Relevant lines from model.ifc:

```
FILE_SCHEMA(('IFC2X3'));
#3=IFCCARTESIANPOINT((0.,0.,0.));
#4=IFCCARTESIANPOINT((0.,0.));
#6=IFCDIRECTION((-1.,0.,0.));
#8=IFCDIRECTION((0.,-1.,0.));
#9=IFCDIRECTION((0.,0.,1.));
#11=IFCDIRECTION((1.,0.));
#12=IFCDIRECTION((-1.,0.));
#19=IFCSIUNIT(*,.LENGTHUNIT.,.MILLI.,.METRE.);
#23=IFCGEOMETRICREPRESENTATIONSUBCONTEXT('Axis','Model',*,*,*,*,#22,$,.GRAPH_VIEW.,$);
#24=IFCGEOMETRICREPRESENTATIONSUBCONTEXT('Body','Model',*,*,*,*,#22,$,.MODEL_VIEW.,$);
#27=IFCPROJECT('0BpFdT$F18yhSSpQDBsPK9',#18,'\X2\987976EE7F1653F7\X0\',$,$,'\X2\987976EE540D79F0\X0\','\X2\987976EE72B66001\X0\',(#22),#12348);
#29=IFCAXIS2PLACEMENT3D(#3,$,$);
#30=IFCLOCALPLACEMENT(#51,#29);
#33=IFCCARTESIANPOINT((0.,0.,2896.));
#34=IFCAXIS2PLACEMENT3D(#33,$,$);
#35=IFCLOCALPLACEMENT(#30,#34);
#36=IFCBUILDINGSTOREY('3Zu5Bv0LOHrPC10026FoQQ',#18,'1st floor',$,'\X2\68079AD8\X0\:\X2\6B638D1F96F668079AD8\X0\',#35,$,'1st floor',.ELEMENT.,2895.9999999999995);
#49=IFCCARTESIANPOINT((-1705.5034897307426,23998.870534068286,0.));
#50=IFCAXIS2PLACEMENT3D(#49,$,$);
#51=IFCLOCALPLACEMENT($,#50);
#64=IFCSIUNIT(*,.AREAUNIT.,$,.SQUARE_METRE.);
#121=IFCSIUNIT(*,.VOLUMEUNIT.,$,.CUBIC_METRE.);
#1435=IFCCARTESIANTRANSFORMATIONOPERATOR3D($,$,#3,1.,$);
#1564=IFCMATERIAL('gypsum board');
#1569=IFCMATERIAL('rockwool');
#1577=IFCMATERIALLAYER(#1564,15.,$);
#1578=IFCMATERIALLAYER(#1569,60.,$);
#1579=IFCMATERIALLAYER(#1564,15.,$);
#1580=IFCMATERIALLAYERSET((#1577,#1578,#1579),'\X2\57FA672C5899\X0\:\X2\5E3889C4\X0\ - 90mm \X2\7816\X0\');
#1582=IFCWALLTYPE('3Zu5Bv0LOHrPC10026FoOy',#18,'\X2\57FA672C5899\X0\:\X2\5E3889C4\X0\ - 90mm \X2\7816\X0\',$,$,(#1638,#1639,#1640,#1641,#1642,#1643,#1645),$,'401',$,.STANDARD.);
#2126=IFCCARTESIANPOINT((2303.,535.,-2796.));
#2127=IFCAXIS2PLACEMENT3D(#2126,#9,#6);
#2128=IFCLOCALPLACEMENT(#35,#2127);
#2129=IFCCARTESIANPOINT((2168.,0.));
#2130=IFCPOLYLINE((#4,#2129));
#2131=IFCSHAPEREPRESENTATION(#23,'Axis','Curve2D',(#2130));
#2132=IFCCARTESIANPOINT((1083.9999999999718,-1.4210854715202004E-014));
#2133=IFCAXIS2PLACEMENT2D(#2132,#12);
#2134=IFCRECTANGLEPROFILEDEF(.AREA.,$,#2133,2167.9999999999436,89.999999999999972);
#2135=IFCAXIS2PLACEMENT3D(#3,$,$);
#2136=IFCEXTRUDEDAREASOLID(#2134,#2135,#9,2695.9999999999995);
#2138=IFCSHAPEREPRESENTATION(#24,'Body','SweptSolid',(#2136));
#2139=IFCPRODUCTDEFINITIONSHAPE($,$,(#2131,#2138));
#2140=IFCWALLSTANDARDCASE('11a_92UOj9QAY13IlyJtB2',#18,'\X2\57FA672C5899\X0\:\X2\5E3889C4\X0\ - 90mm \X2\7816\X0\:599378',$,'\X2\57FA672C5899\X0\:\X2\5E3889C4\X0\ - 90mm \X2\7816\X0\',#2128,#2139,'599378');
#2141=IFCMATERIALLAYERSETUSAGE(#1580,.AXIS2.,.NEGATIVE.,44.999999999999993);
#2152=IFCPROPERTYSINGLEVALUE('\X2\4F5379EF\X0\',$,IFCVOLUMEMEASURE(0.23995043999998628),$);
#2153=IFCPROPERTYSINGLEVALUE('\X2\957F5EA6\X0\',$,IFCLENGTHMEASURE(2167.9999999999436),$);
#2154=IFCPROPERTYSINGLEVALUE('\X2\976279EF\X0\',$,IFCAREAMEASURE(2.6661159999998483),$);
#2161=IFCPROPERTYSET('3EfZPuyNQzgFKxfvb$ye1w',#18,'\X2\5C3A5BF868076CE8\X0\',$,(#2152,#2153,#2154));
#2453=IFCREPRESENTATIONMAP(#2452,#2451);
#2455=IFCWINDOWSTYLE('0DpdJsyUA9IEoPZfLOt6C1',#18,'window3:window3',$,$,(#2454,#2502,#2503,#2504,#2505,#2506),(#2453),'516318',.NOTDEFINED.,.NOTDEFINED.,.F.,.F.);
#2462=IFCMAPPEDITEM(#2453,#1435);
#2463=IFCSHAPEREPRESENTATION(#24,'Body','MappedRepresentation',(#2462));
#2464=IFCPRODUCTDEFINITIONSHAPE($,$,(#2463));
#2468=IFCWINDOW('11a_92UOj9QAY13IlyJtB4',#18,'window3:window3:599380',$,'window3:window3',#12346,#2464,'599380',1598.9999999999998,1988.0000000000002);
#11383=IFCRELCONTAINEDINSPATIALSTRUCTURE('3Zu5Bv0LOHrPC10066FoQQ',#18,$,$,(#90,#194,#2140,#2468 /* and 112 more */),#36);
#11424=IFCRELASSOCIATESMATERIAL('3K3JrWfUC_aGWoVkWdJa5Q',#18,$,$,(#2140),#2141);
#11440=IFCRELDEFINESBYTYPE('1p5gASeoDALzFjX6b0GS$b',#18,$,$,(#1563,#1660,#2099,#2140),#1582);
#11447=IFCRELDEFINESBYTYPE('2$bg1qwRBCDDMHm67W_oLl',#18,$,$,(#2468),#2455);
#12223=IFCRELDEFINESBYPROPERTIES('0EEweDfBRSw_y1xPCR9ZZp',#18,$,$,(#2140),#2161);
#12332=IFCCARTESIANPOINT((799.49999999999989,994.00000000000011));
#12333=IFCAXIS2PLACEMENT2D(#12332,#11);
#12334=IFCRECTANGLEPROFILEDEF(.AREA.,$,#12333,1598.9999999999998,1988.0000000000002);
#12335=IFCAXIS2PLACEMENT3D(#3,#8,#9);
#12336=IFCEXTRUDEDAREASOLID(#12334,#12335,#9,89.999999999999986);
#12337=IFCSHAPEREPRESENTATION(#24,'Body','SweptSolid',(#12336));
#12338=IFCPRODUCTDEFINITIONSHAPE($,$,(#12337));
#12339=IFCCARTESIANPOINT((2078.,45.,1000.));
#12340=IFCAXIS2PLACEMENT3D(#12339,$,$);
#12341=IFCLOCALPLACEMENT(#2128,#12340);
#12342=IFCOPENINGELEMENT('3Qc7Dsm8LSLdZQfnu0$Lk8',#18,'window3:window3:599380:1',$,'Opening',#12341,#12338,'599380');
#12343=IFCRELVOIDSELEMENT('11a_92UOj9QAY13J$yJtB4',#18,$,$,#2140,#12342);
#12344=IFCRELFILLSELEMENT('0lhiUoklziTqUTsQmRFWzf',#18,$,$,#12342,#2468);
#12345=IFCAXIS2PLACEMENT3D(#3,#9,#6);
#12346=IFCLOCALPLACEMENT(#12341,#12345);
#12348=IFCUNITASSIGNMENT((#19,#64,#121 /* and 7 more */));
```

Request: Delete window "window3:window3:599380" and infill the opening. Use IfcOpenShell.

```python
import ifcopenshell
import ifcopenshell.api.feature
import ifcopenshell.api.pset
import ifcopenshell.api.root
import ifcopenshell.geom
import ifcopenshell.util.element
import ifcopenshell.util.shape
import ifcopenshell.util.unit

model = ifcopenshell.open("model.ifc")
area_scale = ifcopenshell.util.unit.calculate_unit_scale(model, "AREAUNIT")
volume_scale = ifcopenshell.util.unit.calculate_unit_scale(model, "VOLUMEUNIT")
settings = ifcopenshell.geom.settings()


def volume(element):
    """Net volume in cubic metres, openings subtracted."""
    shape = ifcopenshell.geom.create_shape(settings, element)
    return ifcopenshell.util.shape.get_volume(shape.geometry)


window = model.by_id(2468)
opening = window.FillsVoids[0].RelatingOpeningElement
wall = opening.VoidsElements[0].RelatingBuildingElement
before = volume(wall)

ifcopenshell.api.root.remove_product(model, product=window)
ifcopenshell.api.feature.remove_feature(model, feature=opening)

after = volume(wall)
thickness = 0.09  # wall thickness in metres

# Update the wall's stored quantities.
pset = model.by_id(ifcopenshell.util.element.get_pset(wall, "尺寸标注", should_inherit=False)["id"])
ifcopenshell.api.pset.edit_pset(model, pset=pset, properties={
    "体积": model.create_entity("IfcVolumeMeasure", after / volume_scale),
    "面积": model.create_entity("IfcAreaMeasure", after / thickness / area_scale),
})

print(f"wall volume {before:.3f} -> {after:.3f} m3")

model.write("model_updated.ifc")
```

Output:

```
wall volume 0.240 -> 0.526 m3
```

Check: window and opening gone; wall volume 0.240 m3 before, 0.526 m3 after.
